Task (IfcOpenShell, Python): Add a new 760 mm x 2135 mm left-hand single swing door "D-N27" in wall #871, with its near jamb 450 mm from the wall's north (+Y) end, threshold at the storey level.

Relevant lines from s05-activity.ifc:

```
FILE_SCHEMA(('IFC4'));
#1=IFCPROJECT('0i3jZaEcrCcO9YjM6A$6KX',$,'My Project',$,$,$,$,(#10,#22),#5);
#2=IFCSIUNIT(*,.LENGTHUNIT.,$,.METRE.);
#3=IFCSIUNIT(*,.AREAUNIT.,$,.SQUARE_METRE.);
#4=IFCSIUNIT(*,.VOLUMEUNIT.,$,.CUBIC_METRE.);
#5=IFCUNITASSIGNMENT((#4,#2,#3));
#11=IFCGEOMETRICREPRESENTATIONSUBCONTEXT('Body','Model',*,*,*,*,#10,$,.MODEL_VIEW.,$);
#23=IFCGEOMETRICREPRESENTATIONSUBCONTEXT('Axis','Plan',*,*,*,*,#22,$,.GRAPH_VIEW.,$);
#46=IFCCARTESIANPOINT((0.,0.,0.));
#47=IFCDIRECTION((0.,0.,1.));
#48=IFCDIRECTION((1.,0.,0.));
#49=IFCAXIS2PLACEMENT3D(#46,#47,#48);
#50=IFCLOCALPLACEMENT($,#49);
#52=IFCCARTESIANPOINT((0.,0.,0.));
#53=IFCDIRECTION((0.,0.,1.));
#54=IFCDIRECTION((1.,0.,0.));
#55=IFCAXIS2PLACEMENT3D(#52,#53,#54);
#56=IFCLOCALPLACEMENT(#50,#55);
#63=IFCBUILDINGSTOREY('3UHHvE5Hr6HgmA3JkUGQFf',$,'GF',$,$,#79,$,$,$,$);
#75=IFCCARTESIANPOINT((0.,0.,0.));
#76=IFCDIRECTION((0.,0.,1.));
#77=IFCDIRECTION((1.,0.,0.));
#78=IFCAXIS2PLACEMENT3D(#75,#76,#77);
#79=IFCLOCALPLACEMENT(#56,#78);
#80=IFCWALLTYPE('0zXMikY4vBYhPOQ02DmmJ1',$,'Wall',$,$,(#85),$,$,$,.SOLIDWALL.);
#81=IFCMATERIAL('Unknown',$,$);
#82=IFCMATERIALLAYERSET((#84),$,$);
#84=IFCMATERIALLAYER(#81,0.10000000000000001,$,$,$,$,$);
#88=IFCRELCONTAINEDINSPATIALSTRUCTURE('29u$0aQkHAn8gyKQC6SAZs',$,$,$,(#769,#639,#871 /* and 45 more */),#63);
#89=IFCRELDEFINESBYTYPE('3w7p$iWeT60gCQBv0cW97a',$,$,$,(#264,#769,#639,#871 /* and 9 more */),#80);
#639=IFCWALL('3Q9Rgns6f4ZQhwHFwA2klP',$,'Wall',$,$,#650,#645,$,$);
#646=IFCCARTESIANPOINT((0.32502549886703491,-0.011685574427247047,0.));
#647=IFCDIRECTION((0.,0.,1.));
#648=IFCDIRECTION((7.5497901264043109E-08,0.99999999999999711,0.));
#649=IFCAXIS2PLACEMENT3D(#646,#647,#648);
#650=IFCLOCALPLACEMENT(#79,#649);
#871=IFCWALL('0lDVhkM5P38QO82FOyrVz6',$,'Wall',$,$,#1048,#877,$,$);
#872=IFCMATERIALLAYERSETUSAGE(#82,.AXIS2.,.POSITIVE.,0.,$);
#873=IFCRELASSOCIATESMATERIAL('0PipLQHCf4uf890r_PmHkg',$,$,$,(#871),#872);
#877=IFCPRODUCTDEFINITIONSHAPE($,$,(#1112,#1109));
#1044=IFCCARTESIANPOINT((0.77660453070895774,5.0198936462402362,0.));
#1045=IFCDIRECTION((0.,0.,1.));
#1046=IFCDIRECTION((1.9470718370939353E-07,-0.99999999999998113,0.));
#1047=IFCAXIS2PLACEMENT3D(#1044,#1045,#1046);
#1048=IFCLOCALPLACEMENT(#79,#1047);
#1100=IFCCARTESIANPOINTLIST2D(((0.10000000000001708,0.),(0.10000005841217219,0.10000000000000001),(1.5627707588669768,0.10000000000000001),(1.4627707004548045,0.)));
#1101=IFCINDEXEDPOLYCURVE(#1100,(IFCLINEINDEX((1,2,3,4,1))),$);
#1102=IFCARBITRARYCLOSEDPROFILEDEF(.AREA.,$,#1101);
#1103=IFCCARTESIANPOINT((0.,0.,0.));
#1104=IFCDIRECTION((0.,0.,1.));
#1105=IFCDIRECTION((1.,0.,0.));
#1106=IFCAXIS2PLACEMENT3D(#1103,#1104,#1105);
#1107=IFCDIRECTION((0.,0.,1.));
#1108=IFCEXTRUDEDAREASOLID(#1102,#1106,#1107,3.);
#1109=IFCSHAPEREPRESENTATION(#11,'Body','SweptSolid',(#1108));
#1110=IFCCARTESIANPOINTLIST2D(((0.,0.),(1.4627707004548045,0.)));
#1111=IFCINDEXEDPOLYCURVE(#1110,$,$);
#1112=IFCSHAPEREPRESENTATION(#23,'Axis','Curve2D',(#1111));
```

```python
import numpy as np
import ifcopenshell
import ifcopenshell.api.feature
import ifcopenshell.api.geometry
import ifcopenshell.api.root
import ifcopenshell.api.spatial
import ifcopenshell.geom
import ifcopenshell.util.element
import ifcopenshell.util.placement
import ifcopenshell.util.representation
import ifcopenshell.util.shape
import ifcopenshell.util.unit

model = ifcopenshell.open("s05-activity.ifc")
unit_scale = ifcopenshell.util.unit.calculate_unit_scale(model)
settings = ifcopenshell.geom.settings()


def volume(element):
    """Net volume in cubic metres, openings subtracted."""
    shape = ifcopenshell.geom.create_shape(settings, element)
    return ifcopenshell.util.shape.get_volume(shape.geometry)


wall = model.by_id(871)
storey = ifcopenshell.util.element.get_container(wall, ifc_class="IfcBuildingStorey")
context = ifcopenshell.util.representation.get_context(model, "Model", "Body", "MODEL_VIEW")
before = volume(wall)

width, height, from_end, sill = 0.76, 2.135, 0.45, 0.0  # metres

# The wall runs along its own X axis, and the end named is its -X end.
wall_shape = ifcopenshell.geom.create_shape(settings, wall)
x, y, z = ifcopenshell.util.shape.get_vertices(wall_shape.geometry).T
start = x.min() + from_end
face, thickness = float(y.min()), float(y.max() - y.min())
wall_matrix = ifcopenshell.util.placement.get_local_placement(wall.ObjectPlacement)
level = ifcopenshell.util.placement.get_local_placement(storey.ObjectPlacement)[2, 3]


def in_wall(x, y):
    """Placement at x, y metres in the wall's axes, at sill height."""
    matrix = wall_matrix.copy()
    matrix[:, 3] = wall_matrix @ np.array([x / unit_scale, y / unit_scale, 0.0, 1.0])
    matrix[2, 3] = level + sill / unit_scale
    return matrix


# Opening: a box that overshoots both wall faces by 50 mm.
opening = ifcopenshell.api.root.create_entity(model, ifc_class="IfcOpeningElement", predefined_type="OPENING")
box = ifcopenshell.api.geometry.add_wall_representation(
    model, context=context, length=width, height=height, thickness=thickness + 0.1
)
ifcopenshell.api.geometry.assign_representation(model, product=opening, representation=box)
ifcopenshell.api.geometry.edit_object_placement(model, product=opening, matrix=in_wall(start, face - 0.05), is_si=False)
ifcopenshell.api.feature.add_feature(model, feature=opening, element=wall)

door = ifcopenshell.api.root.create_entity(model, ifc_class="IfcDoor", name="D-N27", predefined_type="DOOR")
door.OverallWidth, door.OverallHeight = width / unit_scale, height / unit_scale
door.OperationType = "SINGLE_SWING_LEFT"
body = ifcopenshell.api.geometry.add_door_representation(
    model,
    context=context,
    overall_width=door.OverallWidth,
    overall_height=door.OverallHeight,
    operation_type="SINGLE_SWING_LEFT",
    lining_properties={"LiningDepth": thickness / unit_scale, "ThresholdDepth": thickness / unit_scale},
)
ifcopenshell.api.geometry.assign_representation(model, product=door, representation=body)
ifcopenshell.api.spatial.assign_container(model, products=[door], relating_structure=storey)
ifcopenshell.api.feature.add_filling(model, opening=opening, element=door)

# The lining spans the wall, so the door starts at the wall face.
ifcopenshell.api.geometry.edit_object_placement(model, product=door, matrix=in_wall(start, face), is_si=False)

after = volume(wall)

print(f"wall volume {before:.3f} -> {after:.3f} m3")

model.write("s05-activity_updated.ifc")
```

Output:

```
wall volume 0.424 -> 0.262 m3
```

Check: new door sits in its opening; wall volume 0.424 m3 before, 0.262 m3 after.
